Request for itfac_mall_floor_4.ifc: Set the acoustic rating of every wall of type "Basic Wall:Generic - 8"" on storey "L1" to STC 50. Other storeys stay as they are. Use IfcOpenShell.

First a look at what the model holds.

```python
import ifcopenshell
import ifcopenshell.util.element

model = ifcopenshell.open("itfac_mall_floor_4.ifc")
print(model.schema)
storey = next(s for s in model.by_type("IfcBuildingStorey") if s.Name == "L1")
walls = [e for e in ifcopenshell.util.element.get_decomposition(storey) if e.is_a("IfcWall")]
seen = {}
for e in walls:
    element_type = ifcopenshell.util.element.get_type(e)
    key = (element_type.Name if element_type != e and element_type else None, ifcopenshell.util.element.get_pset(e, "Pset_WallCommon", "AcousticRating"))
    seen[key] = seen.get(key, 0) + 1
for (name, value), count in sorted(seen.items(), key=str):
    print(count, "x", name, "|", value)
```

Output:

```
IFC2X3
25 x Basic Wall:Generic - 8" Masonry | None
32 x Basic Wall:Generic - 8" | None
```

```python
import ifcopenshell
import ifcopenshell.api.pset
import ifcopenshell.util.element

model = ifcopenshell.open("itfac_mall_floor_4.ifc")

storey = next(s for s in model.by_type("IfcBuildingStorey") if s.Name == "L1")
walls = [e for e in ifcopenshell.util.element.get_decomposition(storey) if e.is_a("IfcWall")]

count = 0
for e in walls:
    element_type = ifcopenshell.util.element.get_type(e)
    if element_type in (None, e) or element_type.Name != 'Basic Wall:Generic - 8"':
        continue
    # add_pset returns the element's existing set when there is one.
    pset = ifcopenshell.api.pset.add_pset(model, product=e, name="Pset_WallCommon")
    ifcopenshell.api.pset.edit_pset(model, pset=pset, properties={"AcousticRating": "STC 50"})
    count += 1

print(count, "walls updated")

model.write("itfac_mall_floor_4_updated.ifc")
```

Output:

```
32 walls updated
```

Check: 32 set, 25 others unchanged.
